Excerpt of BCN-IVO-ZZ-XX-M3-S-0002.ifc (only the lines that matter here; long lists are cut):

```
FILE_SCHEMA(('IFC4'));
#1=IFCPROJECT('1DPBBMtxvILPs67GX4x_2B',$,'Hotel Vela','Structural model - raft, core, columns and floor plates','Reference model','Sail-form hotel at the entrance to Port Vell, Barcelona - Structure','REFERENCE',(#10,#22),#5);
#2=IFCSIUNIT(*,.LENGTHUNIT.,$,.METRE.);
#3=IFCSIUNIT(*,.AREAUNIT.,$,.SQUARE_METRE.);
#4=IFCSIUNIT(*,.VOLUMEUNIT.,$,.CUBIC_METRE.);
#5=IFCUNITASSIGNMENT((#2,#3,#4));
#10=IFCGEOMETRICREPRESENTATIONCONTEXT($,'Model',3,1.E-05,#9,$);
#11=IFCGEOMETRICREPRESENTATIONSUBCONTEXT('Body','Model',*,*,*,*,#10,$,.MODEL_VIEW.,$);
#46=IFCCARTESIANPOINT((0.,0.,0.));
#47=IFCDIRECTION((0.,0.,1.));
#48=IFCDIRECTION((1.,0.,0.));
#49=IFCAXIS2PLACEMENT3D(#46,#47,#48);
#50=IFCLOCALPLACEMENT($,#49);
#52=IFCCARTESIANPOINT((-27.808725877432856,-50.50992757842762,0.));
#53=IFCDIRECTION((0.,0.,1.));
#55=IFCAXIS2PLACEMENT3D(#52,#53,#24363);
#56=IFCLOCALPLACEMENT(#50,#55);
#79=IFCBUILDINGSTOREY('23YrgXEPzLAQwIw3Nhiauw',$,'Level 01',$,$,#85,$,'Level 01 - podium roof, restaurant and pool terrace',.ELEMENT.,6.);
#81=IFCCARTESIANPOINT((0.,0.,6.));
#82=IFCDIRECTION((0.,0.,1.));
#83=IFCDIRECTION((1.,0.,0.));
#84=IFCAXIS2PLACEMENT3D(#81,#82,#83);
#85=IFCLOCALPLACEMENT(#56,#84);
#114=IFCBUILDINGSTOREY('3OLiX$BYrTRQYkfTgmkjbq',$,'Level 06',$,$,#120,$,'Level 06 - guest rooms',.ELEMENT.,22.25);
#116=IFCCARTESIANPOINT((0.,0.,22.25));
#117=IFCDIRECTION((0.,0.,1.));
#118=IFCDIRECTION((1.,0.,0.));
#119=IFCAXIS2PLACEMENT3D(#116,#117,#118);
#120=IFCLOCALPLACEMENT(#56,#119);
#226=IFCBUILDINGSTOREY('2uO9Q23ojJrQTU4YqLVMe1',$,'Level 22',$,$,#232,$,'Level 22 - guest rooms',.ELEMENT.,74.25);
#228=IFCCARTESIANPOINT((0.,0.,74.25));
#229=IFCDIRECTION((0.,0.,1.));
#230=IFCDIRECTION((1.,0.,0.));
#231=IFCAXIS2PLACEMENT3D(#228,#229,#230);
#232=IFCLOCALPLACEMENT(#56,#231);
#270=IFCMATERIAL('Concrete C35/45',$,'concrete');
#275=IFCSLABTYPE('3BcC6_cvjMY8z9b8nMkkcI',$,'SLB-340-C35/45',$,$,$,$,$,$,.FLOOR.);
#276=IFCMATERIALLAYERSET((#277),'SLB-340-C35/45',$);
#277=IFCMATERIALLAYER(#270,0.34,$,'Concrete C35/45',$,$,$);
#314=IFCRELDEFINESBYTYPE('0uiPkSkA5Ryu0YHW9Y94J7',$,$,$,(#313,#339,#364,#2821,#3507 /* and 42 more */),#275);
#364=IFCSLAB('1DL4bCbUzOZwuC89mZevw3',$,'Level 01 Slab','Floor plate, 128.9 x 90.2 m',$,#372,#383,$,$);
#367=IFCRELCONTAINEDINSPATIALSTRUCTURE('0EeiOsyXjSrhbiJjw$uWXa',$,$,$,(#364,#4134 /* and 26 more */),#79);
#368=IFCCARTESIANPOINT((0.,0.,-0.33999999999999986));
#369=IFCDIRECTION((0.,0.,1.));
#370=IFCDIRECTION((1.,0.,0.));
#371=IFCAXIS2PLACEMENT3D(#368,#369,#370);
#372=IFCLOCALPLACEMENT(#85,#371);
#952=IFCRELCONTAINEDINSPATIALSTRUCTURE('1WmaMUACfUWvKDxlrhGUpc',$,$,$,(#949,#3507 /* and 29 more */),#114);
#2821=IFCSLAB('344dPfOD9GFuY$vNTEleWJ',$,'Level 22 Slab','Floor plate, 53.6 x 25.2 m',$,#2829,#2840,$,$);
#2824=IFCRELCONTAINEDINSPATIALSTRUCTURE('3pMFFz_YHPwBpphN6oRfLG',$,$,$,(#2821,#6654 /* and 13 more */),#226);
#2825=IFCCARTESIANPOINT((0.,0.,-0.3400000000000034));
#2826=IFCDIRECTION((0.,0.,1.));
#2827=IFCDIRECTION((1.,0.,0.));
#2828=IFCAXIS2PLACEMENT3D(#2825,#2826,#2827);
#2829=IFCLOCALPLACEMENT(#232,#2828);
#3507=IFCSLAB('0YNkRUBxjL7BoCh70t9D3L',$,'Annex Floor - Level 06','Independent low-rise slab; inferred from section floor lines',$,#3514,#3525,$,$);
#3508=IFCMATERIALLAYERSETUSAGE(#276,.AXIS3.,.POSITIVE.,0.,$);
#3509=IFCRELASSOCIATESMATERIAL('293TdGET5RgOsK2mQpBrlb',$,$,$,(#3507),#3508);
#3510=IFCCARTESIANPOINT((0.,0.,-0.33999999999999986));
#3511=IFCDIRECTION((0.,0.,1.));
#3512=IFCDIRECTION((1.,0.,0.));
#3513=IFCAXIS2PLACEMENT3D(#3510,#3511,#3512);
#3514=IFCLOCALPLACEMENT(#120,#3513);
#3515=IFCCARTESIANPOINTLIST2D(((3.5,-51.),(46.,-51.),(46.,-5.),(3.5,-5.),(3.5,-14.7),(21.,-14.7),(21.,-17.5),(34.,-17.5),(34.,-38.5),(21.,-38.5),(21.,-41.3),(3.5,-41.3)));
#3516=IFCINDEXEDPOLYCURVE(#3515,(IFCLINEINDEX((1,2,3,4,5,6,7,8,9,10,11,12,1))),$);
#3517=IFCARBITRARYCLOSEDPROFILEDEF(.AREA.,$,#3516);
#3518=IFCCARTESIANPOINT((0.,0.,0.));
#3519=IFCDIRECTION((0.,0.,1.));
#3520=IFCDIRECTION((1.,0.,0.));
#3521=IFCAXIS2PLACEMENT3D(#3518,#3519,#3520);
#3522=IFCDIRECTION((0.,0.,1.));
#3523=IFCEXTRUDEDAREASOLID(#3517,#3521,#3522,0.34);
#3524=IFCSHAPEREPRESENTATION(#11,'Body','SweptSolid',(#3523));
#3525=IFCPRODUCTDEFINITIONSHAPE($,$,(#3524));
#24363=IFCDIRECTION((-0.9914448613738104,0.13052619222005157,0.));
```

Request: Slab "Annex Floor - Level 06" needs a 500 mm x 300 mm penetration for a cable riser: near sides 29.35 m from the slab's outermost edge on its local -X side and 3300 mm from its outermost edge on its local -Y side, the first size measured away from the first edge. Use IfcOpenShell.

```python
import numpy as np
import ifcopenshell
import ifcopenshell.api.feature
import ifcopenshell.api.geometry
import ifcopenshell.api.root
import ifcopenshell.geom
import ifcopenshell.util.placement
import ifcopenshell.util.representation
import ifcopenshell.util.shape
import ifcopenshell.util.unit

model = ifcopenshell.open("BCN-IVO-ZZ-XX-M3-S-0002.ifc")
unit_scale = ifcopenshell.util.unit.calculate_unit_scale(model)
settings = ifcopenshell.geom.settings()


def volume(element):
    """Net volume in cubic metres, openings subtracted."""
    shape = ifcopenshell.geom.create_shape(settings, element)
    return ifcopenshell.util.shape.get_volume(shape.geometry)


slab = model.by_id(3507)
before = volume(slab)

# Extent in the slab's own axes, in metres. The edges named are its -X and -Y sides.
slab_shape = ifcopenshell.geom.create_shape(settings, slab)
vertices = ifcopenshell.util.shape.get_vertices(slab_shape.geometry)
x_min, y_min, bottom = vertices.min(axis=0)
top = vertices[:, 2].max()

opening = ifcopenshell.api.root.create_entity(model, ifc_class="IfcOpeningElement", name="Cable riser opening", predefined_type="OPENING")
context = ifcopenshell.util.representation.get_context(model, "Model", "Body", "MODEL_VIEW")
width, depth = 0.5, 0.3
outline = [(0.0, 0.0), (width, 0.0), (width, depth), (0.0, depth), (0.0, 0.0)]
# Overshoot both faces by 50 mm so the cut is clean.
shape = ifcopenshell.api.geometry.add_slab_representation(
    model, context=context, depth=top - bottom + 0.1, polyline=outline
)
ifcopenshell.api.geometry.assign_representation(model, product=opening, representation=shape)

matrix = ifcopenshell.util.placement.get_local_placement(slab.ObjectPlacement)
matrix[:, 3] = matrix @ np.append(np.array([x_min + 29.35, y_min + 3.3, bottom - 0.05]) / unit_scale, 1.0)
ifcopenshell.api.geometry.edit_object_placement(model, product=opening, matrix=matrix, is_si=False)
ifcopenshell.api.feature.add_feature(model, feature=opening, element=slab)

after = volume(slab)

print(f"slab volume {before:.3f} -> {after:.3f} m3")

model.write("BCN-IVO-ZZ-XX-M3-S-0002_v2.ifc")
```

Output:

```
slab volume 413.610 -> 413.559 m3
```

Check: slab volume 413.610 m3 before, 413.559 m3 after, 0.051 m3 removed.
